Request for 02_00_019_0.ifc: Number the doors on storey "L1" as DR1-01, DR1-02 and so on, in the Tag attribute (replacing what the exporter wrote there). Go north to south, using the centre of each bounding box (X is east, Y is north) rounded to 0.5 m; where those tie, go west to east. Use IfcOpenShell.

First a look at what the model holds.

```python
import ifcopenshell
import ifcopenshell.util.element
import ifcopenshell.util.placement

model = ifcopenshell.open("02_00_019_0.ifc")
print(model.schema)
storey = next(s for s in model.by_type("IfcBuildingStorey") if s.Name == "L1")
doors = [e for e in ifcopenshell.util.element.get_decomposition(storey) if e.is_a("IfcDoor")]
for e in sorted(doors, key=lambda e: e.id()):
    origin = ifcopenshell.util.placement.get_local_placement(e.ObjectPlacement)[:3, 3]
    print(e.id(), e.Tag, e.Name, origin.round(2) + 0.0, sep=" | ")
```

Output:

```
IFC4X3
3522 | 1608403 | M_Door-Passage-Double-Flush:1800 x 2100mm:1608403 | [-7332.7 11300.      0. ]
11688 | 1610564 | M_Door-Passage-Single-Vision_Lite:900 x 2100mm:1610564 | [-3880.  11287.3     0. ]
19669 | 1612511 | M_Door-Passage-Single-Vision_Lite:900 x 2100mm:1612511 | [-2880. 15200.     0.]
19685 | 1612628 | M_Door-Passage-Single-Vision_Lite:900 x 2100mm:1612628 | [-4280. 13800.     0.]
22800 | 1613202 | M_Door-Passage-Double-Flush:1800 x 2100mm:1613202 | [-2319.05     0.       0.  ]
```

```python
import ifcopenshell
import ifcopenshell.geom
import ifcopenshell.util.element
import ifcopenshell.util.shape

model = ifcopenshell.open("02_00_019_0.ifc")
settings = ifcopenshell.geom.settings()
settings.set("use-world-coords", True)


def centre(element):
    shape = ifcopenshell.geom.create_shape(settings, element)
    return ifcopenshell.util.shape.get_bbox_centroid(shape.geometry)


storey = next(s for s in model.by_type("IfcBuildingStorey") if s.Name == "L1")
doors = [e for e in ifcopenshell.util.element.get_decomposition(storey) if e.is_a("IfcDoor")]

# Insertion points can sit at a corner or the storey origin, so sort by the geometry (in metres).
centres = {e: centre(e) for e in doors}
doors.sort(key=lambda e: (-round(centres[e][1] / 0.5), centres[e][0]))

for i, e in enumerate(doors, start=1):
    number = f"DR1-{i:02d}"
    e.Tag = number
    print(e.id(), number)

model.write("02_00_019_0_edited.ifc")
```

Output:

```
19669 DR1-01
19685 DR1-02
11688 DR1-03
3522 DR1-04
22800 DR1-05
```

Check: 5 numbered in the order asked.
